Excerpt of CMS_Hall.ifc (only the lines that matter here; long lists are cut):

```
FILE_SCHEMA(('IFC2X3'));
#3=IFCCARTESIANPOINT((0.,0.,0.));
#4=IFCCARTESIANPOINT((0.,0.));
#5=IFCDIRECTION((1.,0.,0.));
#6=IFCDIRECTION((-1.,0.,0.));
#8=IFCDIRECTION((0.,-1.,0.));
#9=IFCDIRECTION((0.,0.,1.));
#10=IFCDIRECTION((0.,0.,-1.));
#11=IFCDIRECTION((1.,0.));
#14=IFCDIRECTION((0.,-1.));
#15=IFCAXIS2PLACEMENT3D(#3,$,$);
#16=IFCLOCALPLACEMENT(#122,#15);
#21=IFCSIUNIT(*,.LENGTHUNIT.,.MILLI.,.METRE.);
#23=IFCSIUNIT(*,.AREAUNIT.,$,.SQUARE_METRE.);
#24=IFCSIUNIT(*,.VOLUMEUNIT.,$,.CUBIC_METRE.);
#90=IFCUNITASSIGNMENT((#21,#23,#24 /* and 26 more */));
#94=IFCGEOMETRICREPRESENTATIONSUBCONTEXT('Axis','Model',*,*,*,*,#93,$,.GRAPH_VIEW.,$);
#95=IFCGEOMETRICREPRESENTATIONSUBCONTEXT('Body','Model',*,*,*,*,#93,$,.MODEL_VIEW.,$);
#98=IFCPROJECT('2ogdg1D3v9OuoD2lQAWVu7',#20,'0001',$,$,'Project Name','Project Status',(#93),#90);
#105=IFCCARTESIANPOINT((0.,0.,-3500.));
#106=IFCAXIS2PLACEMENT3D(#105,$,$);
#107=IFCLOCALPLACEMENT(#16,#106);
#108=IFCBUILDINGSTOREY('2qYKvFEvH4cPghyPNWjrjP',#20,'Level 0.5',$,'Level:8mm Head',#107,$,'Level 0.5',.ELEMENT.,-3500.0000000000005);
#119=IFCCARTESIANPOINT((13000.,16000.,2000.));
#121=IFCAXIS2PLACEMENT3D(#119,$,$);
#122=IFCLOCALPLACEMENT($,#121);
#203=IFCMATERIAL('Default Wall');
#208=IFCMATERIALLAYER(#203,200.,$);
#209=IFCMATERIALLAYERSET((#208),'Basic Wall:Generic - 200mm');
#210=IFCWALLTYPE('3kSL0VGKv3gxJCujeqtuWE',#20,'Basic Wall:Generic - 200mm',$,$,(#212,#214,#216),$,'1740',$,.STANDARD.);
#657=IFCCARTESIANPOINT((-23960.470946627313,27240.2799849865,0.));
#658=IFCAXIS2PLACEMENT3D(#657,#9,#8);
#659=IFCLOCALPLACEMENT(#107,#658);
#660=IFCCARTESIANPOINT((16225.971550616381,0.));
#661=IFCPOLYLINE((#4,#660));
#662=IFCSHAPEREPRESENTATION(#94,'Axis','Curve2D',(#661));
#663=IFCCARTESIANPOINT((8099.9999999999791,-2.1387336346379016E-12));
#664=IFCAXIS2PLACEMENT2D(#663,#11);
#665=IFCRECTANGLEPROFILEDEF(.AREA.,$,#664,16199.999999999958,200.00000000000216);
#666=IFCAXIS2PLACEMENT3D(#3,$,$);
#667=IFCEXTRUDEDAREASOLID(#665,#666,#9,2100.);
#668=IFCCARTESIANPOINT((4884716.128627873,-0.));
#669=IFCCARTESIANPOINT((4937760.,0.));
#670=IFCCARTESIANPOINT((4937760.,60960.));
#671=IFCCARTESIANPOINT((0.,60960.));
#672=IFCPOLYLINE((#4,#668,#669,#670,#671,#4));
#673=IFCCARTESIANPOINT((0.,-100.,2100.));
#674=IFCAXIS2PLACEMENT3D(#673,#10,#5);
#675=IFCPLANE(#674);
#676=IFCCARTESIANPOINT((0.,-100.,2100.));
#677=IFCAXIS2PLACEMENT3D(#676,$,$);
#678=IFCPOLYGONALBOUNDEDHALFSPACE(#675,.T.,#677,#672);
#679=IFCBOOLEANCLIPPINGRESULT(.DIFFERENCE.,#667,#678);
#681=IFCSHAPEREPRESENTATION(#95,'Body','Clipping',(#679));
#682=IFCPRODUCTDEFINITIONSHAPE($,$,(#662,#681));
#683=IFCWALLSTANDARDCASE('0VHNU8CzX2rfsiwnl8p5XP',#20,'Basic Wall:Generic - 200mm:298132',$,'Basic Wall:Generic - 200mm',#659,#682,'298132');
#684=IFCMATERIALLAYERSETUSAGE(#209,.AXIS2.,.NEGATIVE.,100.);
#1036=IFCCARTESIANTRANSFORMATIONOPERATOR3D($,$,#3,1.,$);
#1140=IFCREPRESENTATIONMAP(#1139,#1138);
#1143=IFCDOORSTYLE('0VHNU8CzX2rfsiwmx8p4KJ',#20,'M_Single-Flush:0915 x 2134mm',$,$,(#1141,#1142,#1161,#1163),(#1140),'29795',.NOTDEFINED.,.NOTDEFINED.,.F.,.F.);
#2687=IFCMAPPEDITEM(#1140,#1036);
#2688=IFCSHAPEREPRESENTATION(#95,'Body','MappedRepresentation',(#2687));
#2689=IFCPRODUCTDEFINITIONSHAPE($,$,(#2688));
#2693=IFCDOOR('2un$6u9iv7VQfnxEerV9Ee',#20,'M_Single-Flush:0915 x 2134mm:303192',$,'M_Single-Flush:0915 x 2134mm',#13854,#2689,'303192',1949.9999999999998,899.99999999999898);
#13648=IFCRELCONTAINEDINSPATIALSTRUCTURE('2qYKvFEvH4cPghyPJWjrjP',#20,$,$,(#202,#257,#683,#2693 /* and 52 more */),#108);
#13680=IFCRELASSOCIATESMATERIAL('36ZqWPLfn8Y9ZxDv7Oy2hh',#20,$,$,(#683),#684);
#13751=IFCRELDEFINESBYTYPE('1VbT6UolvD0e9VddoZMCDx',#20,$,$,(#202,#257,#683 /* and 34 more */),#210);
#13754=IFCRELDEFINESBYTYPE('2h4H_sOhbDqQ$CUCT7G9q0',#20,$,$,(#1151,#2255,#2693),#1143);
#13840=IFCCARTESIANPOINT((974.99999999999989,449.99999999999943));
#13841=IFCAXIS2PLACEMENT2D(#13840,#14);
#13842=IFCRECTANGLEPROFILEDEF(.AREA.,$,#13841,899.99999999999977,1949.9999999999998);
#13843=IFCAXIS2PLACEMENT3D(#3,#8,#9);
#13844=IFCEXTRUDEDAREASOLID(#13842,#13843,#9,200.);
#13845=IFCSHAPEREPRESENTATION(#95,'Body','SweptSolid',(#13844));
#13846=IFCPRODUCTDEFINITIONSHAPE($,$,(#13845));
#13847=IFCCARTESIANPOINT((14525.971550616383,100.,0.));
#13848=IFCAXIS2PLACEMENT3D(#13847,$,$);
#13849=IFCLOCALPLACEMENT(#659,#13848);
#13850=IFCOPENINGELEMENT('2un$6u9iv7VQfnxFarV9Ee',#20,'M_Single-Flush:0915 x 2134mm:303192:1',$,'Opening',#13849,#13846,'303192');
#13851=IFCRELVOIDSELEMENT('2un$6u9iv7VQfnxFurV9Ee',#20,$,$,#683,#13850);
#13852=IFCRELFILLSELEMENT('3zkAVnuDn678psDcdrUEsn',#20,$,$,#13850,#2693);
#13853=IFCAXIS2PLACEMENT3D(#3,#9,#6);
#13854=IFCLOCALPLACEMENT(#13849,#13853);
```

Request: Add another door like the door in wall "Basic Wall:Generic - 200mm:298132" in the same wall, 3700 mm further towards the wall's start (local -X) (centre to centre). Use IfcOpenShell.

```python
import ifcopenshell
import ifcopenshell.api.feature
import ifcopenshell.api.geometry
import ifcopenshell.api.root
import ifcopenshell.geom
import ifcopenshell.util.element
import ifcopenshell.util.placement
import ifcopenshell.util.shape
import ifcopenshell.util.unit

model = ifcopenshell.open("CMS_Hall.ifc")
unit_scale = ifcopenshell.util.unit.calculate_unit_scale(model)
settings = ifcopenshell.geom.settings()


def volume(element):
    """Net volume in cubic metres, openings subtracted."""
    shape = ifcopenshell.geom.create_shape(settings, element)
    return ifcopenshell.util.shape.get_volume(shape.geometry)


def reuse_history(source, copy):
    """copy_class also copies each property set's owner history, people and application; keep the originals."""
    for rel in copy.IsDefinedBy:
        if rel.is_a("IfcRelDefinesByProperties") and (history := rel.RelatingPropertyDefinition.OwnerHistory):
            rel.RelatingPropertyDefinition.OwnerHistory = source.OwnerHistory
            ifcopenshell.util.element.remove_deep2(model, history)


door = model.by_guid("2un$6u9iv7VQfnxEerV9Ee")
opening = door.FillsVoids[0].RelatingOpeningElement
wall = opening.VoidsElements[0].RelatingBuildingElement
before = volume(wall)
shift = ifcopenshell.util.placement.get_local_placement(wall.ObjectPlacement)[:3, 0] * -3.7 / unit_scale

# copy_class copies the void relationship, type, container and properties, but no geometry.
new_opening = ifcopenshell.api.root.copy_class(model, product=opening)
new_opening.Representation = ifcopenshell.util.element.copy_deep(
    model, opening.Representation, exclude=["IfcGeometricRepresentationContext", "IfcRepresentationMap"]
)
new_opening.Name = "M_Single-Flush:0915 x 2134mm"
new_opening.Tag = None
new_door = ifcopenshell.api.root.copy_class(model, product=door)
new_door.Representation = ifcopenshell.util.element.copy_deep(
    model, door.Representation, exclude=["IfcGeometricRepresentationContext", "IfcRepresentationMap"]
)
new_door.Name = "M_Single-Flush:0915 x 2134mm"
new_door.Tag = None
reuse_history(door, new_door)
fills = ifcopenshell.api.feature.add_filling(model, opening=new_opening, element=new_door)
fills.OwnerHistory = new_door.OwnerHistory  # required in IFC2X3

for old, new in ((opening, new_opening), (door, new_door)):
    matrix = ifcopenshell.util.placement.get_local_placement(old.ObjectPlacement)
    matrix[:3, 3] += shift
    ifcopenshell.api.geometry.edit_object_placement(model, product=new, matrix=matrix, is_si=False)

after = volume(wall)

print(f"wall volume {before:.3f} -> {after:.3f} m3")

model.write("CMS_Hall-out.ifc")
```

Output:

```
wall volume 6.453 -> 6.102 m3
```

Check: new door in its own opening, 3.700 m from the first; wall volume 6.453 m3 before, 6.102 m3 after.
